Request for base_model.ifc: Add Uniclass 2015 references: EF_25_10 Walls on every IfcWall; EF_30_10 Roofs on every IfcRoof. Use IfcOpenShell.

First a look at what the model holds.

```python
import ifcopenshell

model = ifcopenshell.open("base_model.ifc")
print(model.schema)
print("classifications:", [c.Name for c in model.by_type("IfcClassification")])
for ifc_class in ("IfcDoor", "IfcRoof", "IfcStair", "IfcWall", "IfcWindow"):
    print(ifc_class, len(model.by_type(ifc_class)))
```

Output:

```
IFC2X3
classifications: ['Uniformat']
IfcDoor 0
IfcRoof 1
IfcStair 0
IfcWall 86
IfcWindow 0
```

```python
import ifcopenshell
import ifcopenshell.api.classification

model = ifcopenshell.open("base_model.ifc")

# IFC2X3 requires Source and Edition and has no link from the project to the system.
system = model.create_entity("IfcClassification", Source="NBS", Edition="2015", Name="Uniclass 2015")

codes = {
    "IfcWall": ("EF_25_10", "Walls"),
    "IfcRoof": ("EF_30_10", "Roofs"),
}
for ifc_class, (code, name) in codes.items():
    products = model.by_type(ifc_class)
    ifcopenshell.api.classification.add_reference(
        model, products=products, classification=system, identification=code, name=name
    )
    print(code, len(products))

model.write("base_model_v2.ifc")
```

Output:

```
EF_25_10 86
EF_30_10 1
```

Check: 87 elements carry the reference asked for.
